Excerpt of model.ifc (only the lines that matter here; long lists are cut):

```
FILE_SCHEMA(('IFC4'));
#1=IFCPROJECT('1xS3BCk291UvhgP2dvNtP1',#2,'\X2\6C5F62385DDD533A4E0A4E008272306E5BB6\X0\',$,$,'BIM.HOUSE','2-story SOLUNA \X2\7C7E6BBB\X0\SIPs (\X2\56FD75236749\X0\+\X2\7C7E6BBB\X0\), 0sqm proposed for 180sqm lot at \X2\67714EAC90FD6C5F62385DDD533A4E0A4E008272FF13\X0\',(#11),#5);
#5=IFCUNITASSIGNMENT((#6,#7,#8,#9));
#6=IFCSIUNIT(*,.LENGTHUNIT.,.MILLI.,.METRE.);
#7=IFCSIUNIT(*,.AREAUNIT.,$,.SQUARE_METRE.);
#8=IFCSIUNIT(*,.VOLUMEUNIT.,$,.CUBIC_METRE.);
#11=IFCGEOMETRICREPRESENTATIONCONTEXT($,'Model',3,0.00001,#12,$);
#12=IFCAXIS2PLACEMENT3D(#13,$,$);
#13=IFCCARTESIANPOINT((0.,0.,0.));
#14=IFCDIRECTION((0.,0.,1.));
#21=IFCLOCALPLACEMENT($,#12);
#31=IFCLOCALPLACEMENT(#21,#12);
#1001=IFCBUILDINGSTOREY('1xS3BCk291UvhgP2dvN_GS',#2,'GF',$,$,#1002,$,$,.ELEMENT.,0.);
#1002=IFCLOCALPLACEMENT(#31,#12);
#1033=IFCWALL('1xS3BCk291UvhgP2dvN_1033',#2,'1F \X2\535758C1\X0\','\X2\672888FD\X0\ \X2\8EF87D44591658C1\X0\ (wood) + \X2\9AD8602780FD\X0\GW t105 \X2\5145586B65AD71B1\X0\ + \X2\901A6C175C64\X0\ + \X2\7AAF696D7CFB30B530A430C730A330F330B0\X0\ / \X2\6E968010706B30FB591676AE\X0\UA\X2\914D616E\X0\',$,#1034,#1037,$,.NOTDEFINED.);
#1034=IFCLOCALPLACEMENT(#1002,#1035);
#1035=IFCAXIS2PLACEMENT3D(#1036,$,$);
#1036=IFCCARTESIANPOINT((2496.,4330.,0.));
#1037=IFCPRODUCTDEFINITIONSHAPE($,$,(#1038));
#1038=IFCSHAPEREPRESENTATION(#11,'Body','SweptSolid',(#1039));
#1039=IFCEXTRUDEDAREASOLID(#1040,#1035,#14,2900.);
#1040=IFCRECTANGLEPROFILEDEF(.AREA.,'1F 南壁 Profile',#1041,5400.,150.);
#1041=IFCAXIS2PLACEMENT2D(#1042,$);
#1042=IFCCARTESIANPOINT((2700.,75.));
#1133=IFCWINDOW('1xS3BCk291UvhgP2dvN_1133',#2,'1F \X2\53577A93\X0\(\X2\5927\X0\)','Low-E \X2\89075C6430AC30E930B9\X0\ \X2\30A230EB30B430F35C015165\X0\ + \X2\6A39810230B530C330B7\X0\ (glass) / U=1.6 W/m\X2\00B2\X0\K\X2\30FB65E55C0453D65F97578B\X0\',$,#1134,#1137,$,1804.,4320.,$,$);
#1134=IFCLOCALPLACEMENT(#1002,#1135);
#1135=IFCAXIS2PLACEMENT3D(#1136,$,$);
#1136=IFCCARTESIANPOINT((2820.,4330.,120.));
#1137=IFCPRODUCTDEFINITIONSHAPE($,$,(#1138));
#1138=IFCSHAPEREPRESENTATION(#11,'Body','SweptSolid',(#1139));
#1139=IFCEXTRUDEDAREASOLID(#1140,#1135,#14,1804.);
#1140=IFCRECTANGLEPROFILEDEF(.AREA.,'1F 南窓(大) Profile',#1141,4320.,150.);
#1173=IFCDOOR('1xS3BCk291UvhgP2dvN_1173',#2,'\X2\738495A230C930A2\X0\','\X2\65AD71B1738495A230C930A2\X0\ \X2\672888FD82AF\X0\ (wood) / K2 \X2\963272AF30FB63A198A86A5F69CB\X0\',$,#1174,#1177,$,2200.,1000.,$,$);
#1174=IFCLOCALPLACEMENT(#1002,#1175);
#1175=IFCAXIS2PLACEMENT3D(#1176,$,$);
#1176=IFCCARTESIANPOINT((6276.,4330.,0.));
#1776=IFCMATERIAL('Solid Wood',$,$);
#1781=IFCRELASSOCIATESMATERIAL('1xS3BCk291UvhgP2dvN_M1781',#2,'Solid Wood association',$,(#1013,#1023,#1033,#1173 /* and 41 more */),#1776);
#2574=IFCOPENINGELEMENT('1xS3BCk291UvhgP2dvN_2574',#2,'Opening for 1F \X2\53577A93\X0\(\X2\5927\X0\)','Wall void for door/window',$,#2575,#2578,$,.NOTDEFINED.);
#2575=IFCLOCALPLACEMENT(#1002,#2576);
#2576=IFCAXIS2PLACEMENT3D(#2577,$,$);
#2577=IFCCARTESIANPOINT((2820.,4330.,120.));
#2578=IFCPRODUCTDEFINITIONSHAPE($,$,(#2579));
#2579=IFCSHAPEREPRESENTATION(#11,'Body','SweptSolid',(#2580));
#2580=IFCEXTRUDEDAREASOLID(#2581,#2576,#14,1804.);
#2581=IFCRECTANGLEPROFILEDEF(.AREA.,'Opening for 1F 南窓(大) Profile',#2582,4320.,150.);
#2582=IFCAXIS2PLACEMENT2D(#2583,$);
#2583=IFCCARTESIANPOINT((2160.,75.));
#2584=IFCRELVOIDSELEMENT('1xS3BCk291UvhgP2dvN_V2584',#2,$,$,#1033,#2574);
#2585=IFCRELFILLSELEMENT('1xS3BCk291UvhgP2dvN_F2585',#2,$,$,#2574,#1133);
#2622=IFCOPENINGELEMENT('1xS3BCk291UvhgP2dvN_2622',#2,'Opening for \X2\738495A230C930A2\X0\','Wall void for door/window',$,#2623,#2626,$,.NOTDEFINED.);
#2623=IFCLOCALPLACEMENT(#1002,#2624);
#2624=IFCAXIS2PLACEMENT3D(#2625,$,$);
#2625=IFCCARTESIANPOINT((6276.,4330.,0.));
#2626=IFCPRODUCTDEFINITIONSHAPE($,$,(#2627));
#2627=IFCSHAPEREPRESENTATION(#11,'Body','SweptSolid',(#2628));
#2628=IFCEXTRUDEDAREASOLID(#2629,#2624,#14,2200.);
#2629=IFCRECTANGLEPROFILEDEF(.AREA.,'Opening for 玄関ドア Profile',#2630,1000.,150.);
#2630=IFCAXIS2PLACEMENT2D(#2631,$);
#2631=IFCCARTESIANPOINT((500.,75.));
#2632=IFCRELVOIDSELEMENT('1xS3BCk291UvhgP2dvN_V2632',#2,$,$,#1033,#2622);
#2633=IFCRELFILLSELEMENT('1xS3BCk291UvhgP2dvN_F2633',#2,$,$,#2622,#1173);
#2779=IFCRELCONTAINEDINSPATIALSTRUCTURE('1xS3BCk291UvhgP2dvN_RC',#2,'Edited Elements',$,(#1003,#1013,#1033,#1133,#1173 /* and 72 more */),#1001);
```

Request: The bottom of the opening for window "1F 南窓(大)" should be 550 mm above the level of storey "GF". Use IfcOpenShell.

```python
import numpy as np
import ifcopenshell
import ifcopenshell.api.geometry
import ifcopenshell.geom
import ifcopenshell.util.element
import ifcopenshell.util.placement
import ifcopenshell.util.shape
import ifcopenshell.util.unit

model = ifcopenshell.open("model.ifc")
unit_scale = ifcopenshell.util.unit.calculate_unit_scale(model)

window = model.by_guid("1xS3BCk291UvhgP2dvN_1133")
opening = window.FillsVoids[0].RelatingOpeningElement
storey = ifcopenshell.util.element.get_container(window, ifc_class="IfcBuildingStorey")
level = ifcopenshell.util.placement.get_local_placement(storey.ObjectPlacement)[2, 3]

# The opening's origin need not be at the sill, so measure its lowest point.
shape = ifcopenshell.geom.create_shape(ifcopenshell.geom.settings(), opening)
bottom = ifcopenshell.util.shape.get_shape_bottom_elevation(shape, shape.geometry) / unit_scale
dz = level + 550.0 - bottom

shift = np.array([0.0, 0.0, dz])
# The window is not placed relative to its opening, so move both.
for product in (opening, window):
    matrix = ifcopenshell.util.placement.get_local_placement(product.ObjectPlacement)
    matrix[:3, 3] += shift
    ifcopenshell.api.geometry.edit_object_placement(model, product=product, matrix=matrix, is_si=False)

print(f"moved by {dz * unit_scale:+.3f} m")

model.write("model-out.ifc")
```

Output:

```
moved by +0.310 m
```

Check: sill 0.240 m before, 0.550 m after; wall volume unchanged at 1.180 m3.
